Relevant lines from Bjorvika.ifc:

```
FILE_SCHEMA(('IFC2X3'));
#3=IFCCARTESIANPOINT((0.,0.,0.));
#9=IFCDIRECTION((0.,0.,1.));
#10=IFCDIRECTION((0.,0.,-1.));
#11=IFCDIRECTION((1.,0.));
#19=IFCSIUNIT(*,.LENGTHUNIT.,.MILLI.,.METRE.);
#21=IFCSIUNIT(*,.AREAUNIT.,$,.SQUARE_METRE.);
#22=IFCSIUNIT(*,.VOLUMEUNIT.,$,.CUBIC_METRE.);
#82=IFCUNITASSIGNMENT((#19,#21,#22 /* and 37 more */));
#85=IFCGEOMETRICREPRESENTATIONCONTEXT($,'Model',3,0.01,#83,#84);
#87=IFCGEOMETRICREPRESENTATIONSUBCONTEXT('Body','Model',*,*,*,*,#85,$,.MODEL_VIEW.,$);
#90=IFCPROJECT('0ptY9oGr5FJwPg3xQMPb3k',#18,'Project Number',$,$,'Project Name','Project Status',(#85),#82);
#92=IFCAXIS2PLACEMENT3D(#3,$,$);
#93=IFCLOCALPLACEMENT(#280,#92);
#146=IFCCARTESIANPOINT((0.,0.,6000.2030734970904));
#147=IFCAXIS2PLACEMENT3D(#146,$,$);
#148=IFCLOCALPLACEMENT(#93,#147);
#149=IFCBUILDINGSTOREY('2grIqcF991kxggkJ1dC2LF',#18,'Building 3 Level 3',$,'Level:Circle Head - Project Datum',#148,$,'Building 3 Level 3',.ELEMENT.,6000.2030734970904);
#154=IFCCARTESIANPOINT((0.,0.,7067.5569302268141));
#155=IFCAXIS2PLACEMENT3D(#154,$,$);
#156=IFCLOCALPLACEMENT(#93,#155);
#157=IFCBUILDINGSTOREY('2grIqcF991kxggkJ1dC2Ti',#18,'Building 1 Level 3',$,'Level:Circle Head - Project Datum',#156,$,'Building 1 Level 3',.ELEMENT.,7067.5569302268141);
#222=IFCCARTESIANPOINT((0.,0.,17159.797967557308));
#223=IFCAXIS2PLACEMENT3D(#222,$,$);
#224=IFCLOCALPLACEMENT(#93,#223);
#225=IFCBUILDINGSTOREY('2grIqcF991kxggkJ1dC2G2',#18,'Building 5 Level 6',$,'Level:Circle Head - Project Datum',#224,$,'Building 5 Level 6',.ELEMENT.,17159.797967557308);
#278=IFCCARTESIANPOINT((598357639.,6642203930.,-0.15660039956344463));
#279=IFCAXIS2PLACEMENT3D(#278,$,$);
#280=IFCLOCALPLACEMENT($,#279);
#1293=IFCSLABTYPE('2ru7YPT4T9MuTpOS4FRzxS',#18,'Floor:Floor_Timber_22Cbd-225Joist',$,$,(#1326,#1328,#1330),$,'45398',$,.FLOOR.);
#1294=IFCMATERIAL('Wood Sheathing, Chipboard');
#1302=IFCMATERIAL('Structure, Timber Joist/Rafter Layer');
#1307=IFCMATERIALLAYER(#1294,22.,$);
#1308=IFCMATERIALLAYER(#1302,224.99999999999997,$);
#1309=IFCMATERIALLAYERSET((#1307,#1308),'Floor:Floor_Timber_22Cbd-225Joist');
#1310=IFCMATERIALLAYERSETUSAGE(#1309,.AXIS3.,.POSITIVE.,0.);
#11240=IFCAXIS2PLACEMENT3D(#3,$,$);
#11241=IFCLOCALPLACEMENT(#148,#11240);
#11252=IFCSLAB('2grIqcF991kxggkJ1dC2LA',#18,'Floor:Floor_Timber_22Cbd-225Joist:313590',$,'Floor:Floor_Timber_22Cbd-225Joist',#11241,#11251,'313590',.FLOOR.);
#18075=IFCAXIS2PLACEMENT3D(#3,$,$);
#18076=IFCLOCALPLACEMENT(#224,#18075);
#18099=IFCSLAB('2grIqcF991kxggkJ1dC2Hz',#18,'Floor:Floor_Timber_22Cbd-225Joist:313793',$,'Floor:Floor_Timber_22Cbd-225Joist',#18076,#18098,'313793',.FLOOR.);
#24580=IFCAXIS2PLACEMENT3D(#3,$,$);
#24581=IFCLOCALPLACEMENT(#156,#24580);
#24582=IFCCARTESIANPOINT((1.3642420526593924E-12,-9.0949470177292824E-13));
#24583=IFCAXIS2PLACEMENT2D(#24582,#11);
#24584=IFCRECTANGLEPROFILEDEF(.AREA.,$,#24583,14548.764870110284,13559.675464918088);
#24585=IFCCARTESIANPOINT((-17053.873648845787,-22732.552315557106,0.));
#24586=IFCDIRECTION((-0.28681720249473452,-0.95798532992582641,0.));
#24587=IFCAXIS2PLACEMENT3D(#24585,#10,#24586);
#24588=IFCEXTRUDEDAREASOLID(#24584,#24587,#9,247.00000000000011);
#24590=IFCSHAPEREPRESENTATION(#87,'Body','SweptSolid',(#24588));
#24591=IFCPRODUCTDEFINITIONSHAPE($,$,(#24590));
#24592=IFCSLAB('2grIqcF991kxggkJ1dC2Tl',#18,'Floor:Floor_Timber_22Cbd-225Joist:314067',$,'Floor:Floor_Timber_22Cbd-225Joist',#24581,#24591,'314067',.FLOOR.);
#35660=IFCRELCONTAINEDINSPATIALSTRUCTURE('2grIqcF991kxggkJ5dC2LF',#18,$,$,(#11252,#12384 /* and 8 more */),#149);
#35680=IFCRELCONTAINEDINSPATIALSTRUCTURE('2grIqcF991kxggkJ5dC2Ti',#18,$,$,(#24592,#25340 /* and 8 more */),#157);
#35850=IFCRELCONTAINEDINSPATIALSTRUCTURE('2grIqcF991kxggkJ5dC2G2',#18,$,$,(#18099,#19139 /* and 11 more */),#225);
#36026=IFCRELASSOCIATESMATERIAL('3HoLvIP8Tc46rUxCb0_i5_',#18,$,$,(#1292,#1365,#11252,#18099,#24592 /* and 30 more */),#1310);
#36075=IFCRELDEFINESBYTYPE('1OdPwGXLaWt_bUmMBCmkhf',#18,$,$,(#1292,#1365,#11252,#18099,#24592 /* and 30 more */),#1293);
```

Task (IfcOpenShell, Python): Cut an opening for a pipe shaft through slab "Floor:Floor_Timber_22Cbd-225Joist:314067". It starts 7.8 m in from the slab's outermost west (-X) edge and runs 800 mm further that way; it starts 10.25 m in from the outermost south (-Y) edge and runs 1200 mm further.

```python
import numpy as np
import ifcopenshell
import ifcopenshell.api.feature
import ifcopenshell.api.geometry
import ifcopenshell.api.root
import ifcopenshell.geom
import ifcopenshell.util.placement
import ifcopenshell.util.representation
import ifcopenshell.util.shape
import ifcopenshell.util.unit

model = ifcopenshell.open("Bjorvika.ifc")
unit_scale = ifcopenshell.util.unit.calculate_unit_scale(model)
settings = ifcopenshell.geom.settings()


def volume(element):
    """Net volume in cubic metres, openings subtracted."""
    shape = ifcopenshell.geom.create_shape(settings, element)
    return ifcopenshell.util.shape.get_volume(shape.geometry)


slab = model.by_id(24592)
before = volume(slab)

# Extent in the slab's own axes, in metres. The edges named are its -X and -Y sides.
slab_shape = ifcopenshell.geom.create_shape(settings, slab)
vertices = ifcopenshell.util.shape.get_vertices(slab_shape.geometry)
x_min, y_min, bottom = vertices.min(axis=0)
top = vertices[:, 2].max()

opening = ifcopenshell.api.root.create_entity(model, ifc_class="IfcOpeningElement", name="Pipe shaft opening")
context = ifcopenshell.util.representation.get_context(model, "Model", "Body", "MODEL_VIEW")
width, depth = 0.8, 1.2
outline = [(0.0, 0.0), (width, 0.0), (width, depth), (0.0, depth), (0.0, 0.0)]
# Overshoot both faces by 50 mm so the cut is clean.
shape = ifcopenshell.api.geometry.add_slab_representation(
    model, context=context, depth=top - bottom + 0.1, polyline=outline
)
ifcopenshell.api.geometry.assign_representation(model, product=opening, representation=shape)

matrix = ifcopenshell.util.placement.get_local_placement(slab.ObjectPlacement)
matrix[:, 3] = matrix @ np.append(np.array([x_min + 7.8, y_min + 10.25, bottom - 0.05]) / unit_scale, 1.0)
ifcopenshell.api.geometry.edit_object_placement(model, product=opening, matrix=matrix, is_si=False)
ifcopenshell.api.feature.add_feature(model, feature=opening, element=slab)

after = volume(slab)

print(f"slab volume {before:.3f} -> {after:.3f} m3")

model.write("Bjorvika_v2.ifc")
```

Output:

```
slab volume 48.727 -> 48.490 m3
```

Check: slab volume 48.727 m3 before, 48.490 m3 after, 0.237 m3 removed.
